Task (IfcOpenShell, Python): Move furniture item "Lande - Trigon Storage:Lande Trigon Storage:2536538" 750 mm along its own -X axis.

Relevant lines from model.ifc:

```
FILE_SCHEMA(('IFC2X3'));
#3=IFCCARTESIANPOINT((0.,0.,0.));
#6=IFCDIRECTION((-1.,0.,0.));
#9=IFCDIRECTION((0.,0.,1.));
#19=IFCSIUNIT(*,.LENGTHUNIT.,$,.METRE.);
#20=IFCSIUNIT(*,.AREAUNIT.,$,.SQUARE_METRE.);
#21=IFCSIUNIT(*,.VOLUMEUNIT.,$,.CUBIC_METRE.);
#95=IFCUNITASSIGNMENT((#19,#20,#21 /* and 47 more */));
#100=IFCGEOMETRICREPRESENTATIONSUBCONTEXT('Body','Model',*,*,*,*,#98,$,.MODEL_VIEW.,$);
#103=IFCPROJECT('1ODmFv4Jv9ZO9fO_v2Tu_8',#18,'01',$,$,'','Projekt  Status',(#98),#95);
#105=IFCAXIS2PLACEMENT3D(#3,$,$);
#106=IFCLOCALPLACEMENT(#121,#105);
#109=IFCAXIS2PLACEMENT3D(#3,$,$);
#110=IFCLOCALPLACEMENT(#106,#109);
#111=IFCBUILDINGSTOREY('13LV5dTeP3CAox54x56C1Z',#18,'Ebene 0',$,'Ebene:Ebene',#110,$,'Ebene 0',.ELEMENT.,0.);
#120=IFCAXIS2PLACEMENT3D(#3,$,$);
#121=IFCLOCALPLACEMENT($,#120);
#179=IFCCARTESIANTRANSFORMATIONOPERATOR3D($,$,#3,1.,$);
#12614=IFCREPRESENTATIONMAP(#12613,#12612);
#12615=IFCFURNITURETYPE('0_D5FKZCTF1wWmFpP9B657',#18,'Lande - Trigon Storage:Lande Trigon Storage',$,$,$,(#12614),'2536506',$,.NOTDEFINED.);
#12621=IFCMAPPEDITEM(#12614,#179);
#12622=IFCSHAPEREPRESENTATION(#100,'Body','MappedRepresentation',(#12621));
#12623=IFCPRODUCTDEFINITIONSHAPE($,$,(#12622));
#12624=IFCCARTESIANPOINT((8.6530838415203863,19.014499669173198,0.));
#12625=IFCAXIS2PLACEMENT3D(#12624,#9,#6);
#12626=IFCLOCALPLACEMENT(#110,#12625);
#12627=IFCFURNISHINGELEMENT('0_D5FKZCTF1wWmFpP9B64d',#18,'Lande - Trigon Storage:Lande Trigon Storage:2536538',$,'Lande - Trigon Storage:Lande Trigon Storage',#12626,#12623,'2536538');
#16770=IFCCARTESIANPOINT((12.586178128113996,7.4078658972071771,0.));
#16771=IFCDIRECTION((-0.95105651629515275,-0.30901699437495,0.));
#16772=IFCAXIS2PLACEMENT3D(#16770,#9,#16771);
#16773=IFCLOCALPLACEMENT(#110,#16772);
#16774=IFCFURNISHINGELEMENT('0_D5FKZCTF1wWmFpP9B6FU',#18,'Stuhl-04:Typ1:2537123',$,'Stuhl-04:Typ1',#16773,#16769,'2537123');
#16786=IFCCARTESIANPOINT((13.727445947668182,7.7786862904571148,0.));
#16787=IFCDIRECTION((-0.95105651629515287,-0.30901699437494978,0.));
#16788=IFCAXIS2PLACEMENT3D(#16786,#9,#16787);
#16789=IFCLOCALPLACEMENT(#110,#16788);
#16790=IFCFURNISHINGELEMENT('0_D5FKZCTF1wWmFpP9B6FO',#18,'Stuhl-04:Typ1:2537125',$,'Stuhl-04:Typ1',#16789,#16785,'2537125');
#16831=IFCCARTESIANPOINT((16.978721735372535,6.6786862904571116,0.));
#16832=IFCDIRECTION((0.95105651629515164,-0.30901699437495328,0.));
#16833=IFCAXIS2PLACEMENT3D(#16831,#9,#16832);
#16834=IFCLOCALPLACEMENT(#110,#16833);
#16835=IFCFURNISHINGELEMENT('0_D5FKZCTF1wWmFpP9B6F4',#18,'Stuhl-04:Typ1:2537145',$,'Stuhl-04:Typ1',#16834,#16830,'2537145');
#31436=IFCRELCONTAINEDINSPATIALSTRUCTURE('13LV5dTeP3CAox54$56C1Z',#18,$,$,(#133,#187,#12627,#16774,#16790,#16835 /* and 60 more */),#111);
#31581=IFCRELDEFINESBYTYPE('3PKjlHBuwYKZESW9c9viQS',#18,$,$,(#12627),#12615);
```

```python
import ifcopenshell
import ifcopenshell.api.geometry
import ifcopenshell.util.placement

model = ifcopenshell.open("model.ifc")

item = model.by_id(12627)
matrix = ifcopenshell.util.placement.get_local_placement(item.ObjectPlacement)
matrix[:3, 3] -= matrix[:3, 0] * 0.75
ifcopenshell.api.geometry.edit_object_placement(model, product=item, matrix=matrix, is_si=False)

print(ifcopenshell.util.placement.get_local_placement(item.ObjectPlacement).round(3) + 0.0)

model.write("model_edited.ifc")
```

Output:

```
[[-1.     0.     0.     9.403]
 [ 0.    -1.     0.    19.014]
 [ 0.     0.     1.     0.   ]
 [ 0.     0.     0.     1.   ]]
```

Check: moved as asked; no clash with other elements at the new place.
